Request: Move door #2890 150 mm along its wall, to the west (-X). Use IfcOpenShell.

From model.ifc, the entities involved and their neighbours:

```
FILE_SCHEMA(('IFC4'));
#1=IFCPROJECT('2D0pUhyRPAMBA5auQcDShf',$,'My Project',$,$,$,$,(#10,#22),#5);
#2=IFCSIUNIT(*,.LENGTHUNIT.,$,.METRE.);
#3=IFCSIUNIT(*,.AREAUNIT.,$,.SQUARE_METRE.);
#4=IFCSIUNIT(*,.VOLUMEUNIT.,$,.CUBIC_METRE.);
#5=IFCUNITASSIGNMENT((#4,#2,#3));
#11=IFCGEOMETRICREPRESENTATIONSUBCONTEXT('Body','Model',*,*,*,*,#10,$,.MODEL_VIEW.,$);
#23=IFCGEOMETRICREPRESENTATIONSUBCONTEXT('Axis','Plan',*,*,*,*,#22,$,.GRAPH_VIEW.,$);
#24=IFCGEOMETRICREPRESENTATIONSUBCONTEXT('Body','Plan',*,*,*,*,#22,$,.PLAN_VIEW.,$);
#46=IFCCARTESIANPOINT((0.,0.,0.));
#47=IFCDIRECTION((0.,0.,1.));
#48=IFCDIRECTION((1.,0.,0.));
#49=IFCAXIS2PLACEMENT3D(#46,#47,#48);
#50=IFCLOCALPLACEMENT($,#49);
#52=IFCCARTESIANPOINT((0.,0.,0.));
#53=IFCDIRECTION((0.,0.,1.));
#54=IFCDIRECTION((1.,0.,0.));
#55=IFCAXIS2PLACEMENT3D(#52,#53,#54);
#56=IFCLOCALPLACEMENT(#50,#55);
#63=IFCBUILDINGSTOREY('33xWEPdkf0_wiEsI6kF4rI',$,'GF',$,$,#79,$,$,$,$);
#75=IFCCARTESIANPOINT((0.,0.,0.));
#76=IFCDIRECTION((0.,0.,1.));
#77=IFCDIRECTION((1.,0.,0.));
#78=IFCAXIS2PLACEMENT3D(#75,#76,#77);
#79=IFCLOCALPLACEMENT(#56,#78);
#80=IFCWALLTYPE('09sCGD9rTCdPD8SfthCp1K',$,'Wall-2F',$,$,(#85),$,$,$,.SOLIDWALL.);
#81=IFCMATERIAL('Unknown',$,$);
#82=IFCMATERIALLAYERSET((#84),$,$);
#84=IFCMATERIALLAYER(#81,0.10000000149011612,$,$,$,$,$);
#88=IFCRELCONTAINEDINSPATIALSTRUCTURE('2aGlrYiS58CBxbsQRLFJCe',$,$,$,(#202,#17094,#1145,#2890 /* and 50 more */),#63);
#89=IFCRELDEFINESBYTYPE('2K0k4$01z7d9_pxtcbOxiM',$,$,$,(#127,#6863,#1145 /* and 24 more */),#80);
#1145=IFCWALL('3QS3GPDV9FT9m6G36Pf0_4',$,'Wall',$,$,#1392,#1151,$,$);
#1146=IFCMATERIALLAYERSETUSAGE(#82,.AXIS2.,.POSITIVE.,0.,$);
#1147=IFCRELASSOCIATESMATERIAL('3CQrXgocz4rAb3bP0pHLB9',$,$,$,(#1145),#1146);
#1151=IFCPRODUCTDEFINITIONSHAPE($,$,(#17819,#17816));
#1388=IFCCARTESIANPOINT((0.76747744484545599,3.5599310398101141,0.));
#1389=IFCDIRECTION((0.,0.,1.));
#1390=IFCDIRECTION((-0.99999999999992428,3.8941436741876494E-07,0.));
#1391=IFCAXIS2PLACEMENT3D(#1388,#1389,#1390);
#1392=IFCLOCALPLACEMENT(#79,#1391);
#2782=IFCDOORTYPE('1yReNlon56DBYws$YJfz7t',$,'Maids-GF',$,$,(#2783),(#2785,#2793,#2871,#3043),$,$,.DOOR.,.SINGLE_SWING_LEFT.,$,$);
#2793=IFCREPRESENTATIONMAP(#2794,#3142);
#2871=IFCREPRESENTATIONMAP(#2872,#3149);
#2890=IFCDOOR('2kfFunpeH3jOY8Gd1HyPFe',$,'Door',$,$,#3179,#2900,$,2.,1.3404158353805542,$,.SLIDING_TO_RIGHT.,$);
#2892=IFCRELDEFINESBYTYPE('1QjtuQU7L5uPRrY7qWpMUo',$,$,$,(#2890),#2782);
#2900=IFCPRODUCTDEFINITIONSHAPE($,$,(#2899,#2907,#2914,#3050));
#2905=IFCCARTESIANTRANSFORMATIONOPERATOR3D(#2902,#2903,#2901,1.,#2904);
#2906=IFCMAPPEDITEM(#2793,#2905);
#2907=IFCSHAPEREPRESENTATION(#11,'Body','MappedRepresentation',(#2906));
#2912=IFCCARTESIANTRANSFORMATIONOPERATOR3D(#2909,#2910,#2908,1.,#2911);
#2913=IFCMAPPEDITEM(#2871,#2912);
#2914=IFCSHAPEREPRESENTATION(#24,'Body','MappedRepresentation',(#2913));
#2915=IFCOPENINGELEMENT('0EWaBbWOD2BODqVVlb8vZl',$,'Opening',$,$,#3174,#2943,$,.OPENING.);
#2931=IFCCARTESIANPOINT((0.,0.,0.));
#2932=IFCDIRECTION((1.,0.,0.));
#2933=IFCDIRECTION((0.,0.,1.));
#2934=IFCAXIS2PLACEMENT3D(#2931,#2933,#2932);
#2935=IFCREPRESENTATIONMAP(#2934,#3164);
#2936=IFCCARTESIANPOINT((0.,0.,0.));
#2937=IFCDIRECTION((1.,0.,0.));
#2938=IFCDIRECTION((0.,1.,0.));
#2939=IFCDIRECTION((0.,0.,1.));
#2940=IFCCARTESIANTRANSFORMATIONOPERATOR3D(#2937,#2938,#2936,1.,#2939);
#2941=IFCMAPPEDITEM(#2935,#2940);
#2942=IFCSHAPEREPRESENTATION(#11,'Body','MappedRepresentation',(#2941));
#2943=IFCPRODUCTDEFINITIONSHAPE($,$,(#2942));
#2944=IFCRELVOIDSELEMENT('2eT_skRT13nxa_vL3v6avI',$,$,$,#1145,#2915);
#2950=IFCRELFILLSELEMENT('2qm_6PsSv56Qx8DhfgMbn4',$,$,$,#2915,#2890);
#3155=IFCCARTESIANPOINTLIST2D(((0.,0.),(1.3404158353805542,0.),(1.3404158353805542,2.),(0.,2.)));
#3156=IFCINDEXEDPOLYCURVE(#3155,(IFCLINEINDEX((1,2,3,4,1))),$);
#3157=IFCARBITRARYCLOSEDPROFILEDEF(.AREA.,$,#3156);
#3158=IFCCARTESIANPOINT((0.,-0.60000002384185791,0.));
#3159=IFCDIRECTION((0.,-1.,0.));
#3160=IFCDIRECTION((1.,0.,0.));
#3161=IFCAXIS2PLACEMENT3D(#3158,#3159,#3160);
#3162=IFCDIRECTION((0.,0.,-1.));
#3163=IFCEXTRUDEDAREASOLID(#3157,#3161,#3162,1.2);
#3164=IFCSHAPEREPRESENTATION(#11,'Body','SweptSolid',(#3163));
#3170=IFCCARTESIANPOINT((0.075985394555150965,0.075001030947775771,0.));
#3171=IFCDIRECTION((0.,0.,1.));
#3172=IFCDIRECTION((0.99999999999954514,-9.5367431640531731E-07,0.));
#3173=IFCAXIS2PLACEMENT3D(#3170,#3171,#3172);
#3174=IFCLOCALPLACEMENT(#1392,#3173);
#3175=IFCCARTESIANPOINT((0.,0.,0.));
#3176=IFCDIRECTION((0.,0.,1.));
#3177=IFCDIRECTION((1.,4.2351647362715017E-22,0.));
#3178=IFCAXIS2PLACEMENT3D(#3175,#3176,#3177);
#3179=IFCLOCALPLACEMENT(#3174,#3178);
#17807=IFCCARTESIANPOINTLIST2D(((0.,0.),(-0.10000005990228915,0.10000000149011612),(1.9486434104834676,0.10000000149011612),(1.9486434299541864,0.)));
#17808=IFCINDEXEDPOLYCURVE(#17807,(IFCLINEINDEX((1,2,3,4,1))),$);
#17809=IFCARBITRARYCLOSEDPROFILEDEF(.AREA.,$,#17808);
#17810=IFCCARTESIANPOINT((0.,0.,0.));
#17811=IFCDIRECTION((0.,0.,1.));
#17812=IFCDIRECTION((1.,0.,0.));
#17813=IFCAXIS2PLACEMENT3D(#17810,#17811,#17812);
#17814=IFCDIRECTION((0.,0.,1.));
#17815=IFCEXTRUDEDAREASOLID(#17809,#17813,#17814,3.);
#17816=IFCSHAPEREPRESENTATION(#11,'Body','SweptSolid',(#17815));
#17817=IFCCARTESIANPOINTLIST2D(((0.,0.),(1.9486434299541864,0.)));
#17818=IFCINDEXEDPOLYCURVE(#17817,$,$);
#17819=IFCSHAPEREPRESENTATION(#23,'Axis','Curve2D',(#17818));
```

```python
import ifcopenshell
import ifcopenshell.api.geometry
import ifcopenshell.util.placement
import ifcopenshell.util.unit

model = ifcopenshell.open("model.ifc")
unit_scale = ifcopenshell.util.unit.calculate_unit_scale(model)

door = model.by_guid("2kfFunpeH3jOY8Gd1HyPFe")
opening = door.FillsVoids[0].RelatingOpeningElement
wall = opening.VoidsElements[0].RelatingBuildingElement

wall_matrix = ifcopenshell.util.placement.get_local_placement(wall.ObjectPlacement)
shift = wall_matrix[:3, 0] * 0.15 / unit_scale
before = ifcopenshell.util.placement.get_local_placement(door.ObjectPlacement)[:3, 3].copy()

# The door is placed relative to its opening, so it follows when the opening moves.
matrix = ifcopenshell.util.placement.get_local_placement(opening.ObjectPlacement)
matrix[:3, 3] += shift
ifcopenshell.api.geometry.edit_object_placement(
    model, product=opening, matrix=matrix, is_si=False, should_transform_children=True
)

after = ifcopenshell.util.placement.get_local_placement(door.ObjectPlacement)[:3, 3]
print("door moved by", (after - before).round(3) + 0.0)

model.write("model_updated.ifc")
```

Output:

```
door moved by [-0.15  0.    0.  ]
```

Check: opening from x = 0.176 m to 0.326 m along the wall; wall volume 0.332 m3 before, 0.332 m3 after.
